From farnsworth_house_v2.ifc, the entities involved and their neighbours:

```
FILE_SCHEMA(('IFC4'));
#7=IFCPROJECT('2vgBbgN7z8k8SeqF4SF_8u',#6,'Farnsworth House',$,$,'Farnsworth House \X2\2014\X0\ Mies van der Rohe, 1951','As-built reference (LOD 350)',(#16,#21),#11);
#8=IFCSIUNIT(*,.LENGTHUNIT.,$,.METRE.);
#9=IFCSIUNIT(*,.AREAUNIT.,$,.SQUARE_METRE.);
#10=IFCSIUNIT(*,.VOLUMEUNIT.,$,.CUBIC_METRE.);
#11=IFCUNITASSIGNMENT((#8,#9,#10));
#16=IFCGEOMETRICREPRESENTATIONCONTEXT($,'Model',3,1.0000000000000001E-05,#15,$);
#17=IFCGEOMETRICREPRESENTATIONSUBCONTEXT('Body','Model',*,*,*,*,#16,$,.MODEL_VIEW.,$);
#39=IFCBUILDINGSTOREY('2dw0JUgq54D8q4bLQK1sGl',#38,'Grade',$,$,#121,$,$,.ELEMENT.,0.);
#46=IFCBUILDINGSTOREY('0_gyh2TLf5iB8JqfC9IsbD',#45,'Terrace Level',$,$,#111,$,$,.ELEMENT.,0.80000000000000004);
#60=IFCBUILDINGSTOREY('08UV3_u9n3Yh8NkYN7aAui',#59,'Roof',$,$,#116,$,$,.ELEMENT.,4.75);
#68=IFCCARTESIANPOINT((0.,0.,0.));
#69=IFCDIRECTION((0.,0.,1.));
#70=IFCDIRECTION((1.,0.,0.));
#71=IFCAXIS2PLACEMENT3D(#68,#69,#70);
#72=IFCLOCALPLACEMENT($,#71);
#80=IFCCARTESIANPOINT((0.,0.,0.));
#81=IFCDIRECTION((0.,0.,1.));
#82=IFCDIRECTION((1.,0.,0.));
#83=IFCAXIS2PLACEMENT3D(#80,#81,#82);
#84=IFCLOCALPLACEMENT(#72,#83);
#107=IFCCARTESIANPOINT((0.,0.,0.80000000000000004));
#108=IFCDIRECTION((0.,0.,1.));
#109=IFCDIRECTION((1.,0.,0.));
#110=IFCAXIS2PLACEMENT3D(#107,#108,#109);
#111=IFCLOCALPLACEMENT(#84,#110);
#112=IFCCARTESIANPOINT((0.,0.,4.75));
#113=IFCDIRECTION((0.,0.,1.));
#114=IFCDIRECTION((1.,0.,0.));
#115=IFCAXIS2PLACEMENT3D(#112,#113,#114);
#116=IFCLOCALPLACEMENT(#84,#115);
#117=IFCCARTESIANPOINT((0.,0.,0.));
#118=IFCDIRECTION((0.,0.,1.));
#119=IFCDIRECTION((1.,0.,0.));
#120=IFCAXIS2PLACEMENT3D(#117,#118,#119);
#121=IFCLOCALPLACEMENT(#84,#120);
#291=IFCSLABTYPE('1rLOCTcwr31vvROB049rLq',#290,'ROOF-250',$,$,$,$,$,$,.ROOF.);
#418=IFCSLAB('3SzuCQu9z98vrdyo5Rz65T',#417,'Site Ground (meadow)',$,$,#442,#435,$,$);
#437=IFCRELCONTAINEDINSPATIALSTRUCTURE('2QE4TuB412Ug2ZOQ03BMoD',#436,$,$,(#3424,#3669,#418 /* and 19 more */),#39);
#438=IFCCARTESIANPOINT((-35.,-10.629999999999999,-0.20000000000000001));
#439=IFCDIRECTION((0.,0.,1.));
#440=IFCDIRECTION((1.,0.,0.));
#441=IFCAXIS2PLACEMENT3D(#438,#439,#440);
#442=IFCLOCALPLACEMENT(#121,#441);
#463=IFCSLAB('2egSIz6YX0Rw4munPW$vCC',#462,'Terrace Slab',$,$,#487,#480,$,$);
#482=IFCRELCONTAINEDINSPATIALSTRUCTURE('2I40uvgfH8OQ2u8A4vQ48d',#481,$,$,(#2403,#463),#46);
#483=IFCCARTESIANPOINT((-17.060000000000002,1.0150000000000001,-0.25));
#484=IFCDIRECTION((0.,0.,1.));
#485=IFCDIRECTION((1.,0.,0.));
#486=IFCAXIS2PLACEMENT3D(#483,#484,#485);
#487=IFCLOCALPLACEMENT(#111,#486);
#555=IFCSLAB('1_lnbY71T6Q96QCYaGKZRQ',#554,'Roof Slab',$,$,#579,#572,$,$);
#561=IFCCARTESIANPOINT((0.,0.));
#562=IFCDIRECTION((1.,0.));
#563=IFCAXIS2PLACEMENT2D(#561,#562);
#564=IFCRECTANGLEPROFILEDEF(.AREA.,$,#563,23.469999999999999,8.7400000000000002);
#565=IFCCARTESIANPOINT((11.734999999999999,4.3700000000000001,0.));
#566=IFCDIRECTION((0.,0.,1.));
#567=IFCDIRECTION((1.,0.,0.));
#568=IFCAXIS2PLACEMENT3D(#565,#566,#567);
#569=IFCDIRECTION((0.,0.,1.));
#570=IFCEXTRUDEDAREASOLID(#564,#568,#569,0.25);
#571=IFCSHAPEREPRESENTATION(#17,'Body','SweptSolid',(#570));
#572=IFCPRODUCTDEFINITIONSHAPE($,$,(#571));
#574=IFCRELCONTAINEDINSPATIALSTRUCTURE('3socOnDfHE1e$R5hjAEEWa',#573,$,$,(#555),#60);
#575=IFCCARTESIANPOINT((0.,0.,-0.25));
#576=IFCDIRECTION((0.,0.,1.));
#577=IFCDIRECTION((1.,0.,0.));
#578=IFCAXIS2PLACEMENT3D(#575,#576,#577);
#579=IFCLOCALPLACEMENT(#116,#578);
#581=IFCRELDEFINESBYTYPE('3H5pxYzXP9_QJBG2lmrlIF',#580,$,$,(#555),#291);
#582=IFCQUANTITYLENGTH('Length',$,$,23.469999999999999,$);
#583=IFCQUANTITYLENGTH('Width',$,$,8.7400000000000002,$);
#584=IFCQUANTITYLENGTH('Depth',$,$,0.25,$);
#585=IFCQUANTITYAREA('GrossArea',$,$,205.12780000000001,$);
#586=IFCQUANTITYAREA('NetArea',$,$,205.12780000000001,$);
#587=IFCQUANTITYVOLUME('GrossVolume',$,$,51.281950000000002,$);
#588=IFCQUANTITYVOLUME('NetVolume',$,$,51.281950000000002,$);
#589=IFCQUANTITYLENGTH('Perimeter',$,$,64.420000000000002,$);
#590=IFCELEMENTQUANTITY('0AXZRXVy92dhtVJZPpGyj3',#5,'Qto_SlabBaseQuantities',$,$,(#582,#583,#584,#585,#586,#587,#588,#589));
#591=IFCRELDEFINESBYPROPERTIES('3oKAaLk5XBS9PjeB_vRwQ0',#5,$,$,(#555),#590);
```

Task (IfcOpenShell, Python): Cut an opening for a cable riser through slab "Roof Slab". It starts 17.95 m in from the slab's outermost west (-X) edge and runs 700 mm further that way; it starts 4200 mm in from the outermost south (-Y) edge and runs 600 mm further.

```python
import numpy as np
import ifcopenshell
import ifcopenshell.api.feature
import ifcopenshell.api.geometry
import ifcopenshell.api.pset
import ifcopenshell.api.root
import ifcopenshell.geom
import ifcopenshell.util.element
import ifcopenshell.util.placement
import ifcopenshell.util.representation
import ifcopenshell.util.shape
import ifcopenshell.util.unit

model = ifcopenshell.open("farnsworth_house_v2.ifc")
unit_scale = ifcopenshell.util.unit.calculate_unit_scale(model)
area_scale = ifcopenshell.util.unit.calculate_unit_scale(model, "AREAUNIT")
volume_scale = ifcopenshell.util.unit.calculate_unit_scale(model, "VOLUMEUNIT")
settings = ifcopenshell.geom.settings()


def volume(element):
    """Net volume in cubic metres, openings subtracted."""
    shape = ifcopenshell.geom.create_shape(settings, element)
    return ifcopenshell.util.shape.get_volume(shape.geometry)


slab = model.by_guid("1_lnbY71T6Q96QCYaGKZRQ")
before = volume(slab)

# Extent in the slab's own axes, in metres. The edges named are its -X and -Y sides.
slab_shape = ifcopenshell.geom.create_shape(settings, slab)
vertices = ifcopenshell.util.shape.get_vertices(slab_shape.geometry)
x_min, y_min, bottom = vertices.min(axis=0)
top = vertices[:, 2].max()

opening = ifcopenshell.api.root.create_entity(model, ifc_class="IfcOpeningElement", name="Cable riser opening", predefined_type="OPENING")
context = ifcopenshell.util.representation.get_context(model, "Model", "Body", "MODEL_VIEW")
width, depth = 0.7, 0.6
outline = [(0.0, 0.0), (width, 0.0), (width, depth), (0.0, depth), (0.0, 0.0)]
# Overshoot both faces by 50 mm so the cut is clean.
shape = ifcopenshell.api.geometry.add_slab_representation(
    model, context=context, depth=top - bottom + 0.1, polyline=outline
)
ifcopenshell.api.geometry.assign_representation(model, product=opening, representation=shape)

matrix = ifcopenshell.util.placement.get_local_placement(slab.ObjectPlacement)
matrix[:, 3] = matrix @ np.append(np.array([x_min + 17.95, y_min + 4.2, bottom - 0.05]) / unit_scale, 1.0)
ifcopenshell.api.geometry.edit_object_placement(model, product=opening, matrix=matrix, is_si=False)
ifcopenshell.api.feature.add_feature(model, feature=opening, element=slab)

after = volume(slab)

# Update the slab's stored quantities.
qto = model.by_id(ifcopenshell.util.element.get_pset(slab, "Qto_SlabBaseQuantities", should_inherit=False)["id"])
ifcopenshell.api.pset.edit_qto(model, qto=qto, properties={
    "NetArea": after / (top - bottom) / area_scale,
    "NetVolume": after / volume_scale,
})

print(f"slab volume {before:.3f} -> {after:.3f} m3")

model.write("farnsworth_house_v2-out.ifc")
```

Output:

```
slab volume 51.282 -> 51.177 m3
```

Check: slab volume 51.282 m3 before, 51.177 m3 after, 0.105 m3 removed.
